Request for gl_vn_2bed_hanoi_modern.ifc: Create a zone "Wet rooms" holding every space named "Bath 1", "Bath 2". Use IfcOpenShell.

First a look at what the model holds.

```python
import ifcopenshell

model = ifcopenshell.open("gl_vn_2bed_hanoi_modern.ifc")
print(model.schema)
seen = {}
for space in model.by_type("IfcSpace"):
    seen[space.LongName] = seen.get(space.LongName, 0) + 1
for name, count in sorted(seen.items(), key=str):
    print(count, "x", name)
print("zones:", [z.Name for z in model.by_type("IfcZone")][:20])
```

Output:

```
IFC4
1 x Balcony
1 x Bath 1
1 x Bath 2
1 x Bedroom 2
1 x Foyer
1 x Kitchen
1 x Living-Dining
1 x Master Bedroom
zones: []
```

```python
import ifcopenshell
import ifcopenshell.api.group
import ifcopenshell.api.root

model = ifcopenshell.open("gl_vn_2bed_hanoi_modern.ifc")

names = {"Bath 1", "Bath 2"}
spaces = [s for s in model.by_type("IfcSpace") if s.LongName in names]

zone = ifcopenshell.api.root.create_entity(model, ifc_class="IfcZone", name="Wet rooms")
ifcopenshell.api.group.assign_group(model, products=spaces, group=zone)
print(len(spaces), "spaces in", zone.Name)

model.write("gl_vn_2bed_hanoi_modern_edited.ifc")
```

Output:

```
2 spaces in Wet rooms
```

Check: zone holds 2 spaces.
